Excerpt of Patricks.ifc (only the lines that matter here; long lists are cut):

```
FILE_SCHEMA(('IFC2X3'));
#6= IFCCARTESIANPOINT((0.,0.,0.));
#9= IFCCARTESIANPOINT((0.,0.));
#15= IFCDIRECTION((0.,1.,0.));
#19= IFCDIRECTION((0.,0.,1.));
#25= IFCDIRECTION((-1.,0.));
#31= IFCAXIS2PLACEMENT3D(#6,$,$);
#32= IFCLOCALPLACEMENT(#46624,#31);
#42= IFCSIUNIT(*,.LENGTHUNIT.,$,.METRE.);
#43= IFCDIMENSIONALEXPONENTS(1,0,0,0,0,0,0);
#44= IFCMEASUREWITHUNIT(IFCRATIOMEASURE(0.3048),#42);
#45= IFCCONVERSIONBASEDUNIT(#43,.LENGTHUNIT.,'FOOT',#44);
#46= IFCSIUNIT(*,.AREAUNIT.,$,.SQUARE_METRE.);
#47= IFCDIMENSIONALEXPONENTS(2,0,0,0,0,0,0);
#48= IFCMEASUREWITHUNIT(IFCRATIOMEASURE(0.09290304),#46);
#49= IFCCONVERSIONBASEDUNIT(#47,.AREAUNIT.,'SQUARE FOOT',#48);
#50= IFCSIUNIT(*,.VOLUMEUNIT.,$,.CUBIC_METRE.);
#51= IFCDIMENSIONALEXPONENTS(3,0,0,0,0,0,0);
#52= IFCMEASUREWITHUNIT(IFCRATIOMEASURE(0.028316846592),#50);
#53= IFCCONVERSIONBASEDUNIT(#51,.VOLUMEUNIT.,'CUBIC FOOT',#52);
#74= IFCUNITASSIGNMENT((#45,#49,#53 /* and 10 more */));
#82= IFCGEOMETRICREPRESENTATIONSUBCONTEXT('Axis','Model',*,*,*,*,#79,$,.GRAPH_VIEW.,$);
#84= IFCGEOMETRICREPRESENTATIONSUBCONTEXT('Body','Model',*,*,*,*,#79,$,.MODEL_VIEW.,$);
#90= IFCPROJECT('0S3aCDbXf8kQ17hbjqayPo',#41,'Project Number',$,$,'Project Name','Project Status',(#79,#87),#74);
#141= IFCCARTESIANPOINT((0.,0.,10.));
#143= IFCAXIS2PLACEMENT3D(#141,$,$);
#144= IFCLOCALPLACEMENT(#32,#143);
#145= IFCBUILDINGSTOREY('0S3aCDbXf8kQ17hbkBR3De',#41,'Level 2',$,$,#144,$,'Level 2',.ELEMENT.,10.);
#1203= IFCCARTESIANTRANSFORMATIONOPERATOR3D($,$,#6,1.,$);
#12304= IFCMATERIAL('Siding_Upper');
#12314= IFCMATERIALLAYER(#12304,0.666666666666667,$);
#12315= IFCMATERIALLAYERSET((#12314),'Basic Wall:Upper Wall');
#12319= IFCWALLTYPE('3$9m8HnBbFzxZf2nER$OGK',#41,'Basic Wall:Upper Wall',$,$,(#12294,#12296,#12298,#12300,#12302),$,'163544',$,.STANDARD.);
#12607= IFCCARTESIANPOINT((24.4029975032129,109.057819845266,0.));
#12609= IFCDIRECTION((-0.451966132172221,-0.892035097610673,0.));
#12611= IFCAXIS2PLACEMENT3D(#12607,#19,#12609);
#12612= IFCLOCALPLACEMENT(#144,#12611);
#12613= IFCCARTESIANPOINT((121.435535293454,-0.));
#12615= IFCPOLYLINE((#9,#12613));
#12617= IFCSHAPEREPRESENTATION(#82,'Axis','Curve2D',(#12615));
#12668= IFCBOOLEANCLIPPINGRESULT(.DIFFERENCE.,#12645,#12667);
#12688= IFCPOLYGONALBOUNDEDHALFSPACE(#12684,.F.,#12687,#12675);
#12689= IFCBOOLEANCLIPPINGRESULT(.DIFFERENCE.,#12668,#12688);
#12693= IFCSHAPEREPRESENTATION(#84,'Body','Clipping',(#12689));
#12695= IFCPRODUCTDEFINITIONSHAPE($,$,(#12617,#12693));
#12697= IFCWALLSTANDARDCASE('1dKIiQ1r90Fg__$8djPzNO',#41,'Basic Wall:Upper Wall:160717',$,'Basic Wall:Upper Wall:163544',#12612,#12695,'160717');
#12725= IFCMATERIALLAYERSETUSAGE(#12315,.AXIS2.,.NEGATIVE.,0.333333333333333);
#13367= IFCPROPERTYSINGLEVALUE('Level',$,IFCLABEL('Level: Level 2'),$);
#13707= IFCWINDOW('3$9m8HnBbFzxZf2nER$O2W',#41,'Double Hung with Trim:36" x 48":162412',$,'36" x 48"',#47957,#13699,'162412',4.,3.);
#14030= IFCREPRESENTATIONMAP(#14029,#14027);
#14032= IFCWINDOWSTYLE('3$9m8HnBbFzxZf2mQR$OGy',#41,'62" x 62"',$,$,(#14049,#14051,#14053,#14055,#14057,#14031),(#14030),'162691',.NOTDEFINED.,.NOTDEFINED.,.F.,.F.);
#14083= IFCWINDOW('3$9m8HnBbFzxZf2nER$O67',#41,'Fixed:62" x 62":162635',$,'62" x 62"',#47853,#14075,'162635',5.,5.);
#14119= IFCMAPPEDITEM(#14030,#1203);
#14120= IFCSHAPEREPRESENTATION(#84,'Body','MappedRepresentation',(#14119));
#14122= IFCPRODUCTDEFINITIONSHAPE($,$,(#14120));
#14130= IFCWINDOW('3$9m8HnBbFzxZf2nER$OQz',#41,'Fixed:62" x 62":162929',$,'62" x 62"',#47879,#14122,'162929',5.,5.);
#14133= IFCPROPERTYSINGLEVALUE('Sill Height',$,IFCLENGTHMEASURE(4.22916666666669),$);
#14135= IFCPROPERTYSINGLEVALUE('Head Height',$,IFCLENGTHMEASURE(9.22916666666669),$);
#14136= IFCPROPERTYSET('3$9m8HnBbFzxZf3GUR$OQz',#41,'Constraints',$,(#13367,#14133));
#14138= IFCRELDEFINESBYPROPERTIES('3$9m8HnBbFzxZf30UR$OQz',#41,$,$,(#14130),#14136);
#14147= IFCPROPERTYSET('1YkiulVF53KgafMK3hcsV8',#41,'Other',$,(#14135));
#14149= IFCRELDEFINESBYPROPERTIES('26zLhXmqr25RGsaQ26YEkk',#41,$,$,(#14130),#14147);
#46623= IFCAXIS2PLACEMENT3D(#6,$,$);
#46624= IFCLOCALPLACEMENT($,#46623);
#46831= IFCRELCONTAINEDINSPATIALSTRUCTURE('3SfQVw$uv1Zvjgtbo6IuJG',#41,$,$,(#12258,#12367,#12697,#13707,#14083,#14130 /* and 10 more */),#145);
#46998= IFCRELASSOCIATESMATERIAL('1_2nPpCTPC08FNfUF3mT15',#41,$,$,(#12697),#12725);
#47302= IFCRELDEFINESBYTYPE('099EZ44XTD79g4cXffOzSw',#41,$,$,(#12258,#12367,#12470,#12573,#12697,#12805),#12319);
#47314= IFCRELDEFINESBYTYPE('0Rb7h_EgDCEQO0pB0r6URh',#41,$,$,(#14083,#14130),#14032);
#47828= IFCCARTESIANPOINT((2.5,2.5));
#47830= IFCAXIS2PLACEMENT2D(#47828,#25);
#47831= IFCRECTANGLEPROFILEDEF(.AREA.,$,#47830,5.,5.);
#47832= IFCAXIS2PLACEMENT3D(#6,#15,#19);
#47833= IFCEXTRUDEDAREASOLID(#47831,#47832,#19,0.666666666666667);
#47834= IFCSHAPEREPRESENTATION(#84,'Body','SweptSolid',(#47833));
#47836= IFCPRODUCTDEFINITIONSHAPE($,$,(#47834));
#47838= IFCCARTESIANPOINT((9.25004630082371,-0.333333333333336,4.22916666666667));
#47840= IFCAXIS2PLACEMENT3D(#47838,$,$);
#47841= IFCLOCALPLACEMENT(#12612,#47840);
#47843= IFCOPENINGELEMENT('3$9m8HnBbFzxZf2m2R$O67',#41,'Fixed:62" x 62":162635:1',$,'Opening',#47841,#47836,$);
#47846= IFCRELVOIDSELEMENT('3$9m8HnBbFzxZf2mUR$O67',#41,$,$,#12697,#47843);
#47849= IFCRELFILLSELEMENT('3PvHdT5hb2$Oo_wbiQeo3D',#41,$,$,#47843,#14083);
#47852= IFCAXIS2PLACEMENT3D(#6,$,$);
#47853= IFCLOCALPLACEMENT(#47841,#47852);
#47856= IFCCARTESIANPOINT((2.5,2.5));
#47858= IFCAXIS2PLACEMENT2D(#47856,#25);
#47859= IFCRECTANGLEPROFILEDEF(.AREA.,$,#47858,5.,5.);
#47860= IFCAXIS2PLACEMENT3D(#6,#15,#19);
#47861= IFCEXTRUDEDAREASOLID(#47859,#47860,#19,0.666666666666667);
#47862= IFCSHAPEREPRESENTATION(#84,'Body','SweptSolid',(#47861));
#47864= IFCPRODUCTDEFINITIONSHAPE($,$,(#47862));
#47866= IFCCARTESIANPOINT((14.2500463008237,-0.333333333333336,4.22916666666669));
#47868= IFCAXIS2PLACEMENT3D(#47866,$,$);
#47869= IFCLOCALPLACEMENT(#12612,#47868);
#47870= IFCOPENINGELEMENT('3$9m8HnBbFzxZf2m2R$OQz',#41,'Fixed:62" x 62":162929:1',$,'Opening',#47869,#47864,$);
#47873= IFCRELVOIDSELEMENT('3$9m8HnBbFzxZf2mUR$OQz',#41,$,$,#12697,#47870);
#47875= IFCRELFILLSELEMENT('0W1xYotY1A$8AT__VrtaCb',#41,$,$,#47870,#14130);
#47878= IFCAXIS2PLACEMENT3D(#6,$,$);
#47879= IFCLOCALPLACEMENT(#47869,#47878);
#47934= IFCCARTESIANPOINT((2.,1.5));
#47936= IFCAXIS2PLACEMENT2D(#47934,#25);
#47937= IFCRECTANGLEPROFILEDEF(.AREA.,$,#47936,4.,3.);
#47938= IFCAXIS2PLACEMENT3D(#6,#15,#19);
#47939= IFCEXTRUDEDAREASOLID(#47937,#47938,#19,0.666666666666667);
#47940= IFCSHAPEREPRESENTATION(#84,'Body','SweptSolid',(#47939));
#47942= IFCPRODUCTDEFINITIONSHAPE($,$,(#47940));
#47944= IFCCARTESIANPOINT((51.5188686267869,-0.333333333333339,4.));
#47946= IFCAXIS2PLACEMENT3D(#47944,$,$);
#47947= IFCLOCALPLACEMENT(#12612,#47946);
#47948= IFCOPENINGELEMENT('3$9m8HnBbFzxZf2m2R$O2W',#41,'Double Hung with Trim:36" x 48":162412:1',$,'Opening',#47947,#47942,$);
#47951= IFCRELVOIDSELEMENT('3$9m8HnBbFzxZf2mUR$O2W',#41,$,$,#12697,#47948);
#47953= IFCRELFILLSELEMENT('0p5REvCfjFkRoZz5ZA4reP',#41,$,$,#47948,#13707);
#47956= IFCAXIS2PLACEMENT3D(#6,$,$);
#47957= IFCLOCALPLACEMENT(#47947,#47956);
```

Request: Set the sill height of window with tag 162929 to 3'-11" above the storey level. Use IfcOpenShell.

```python
import numpy as np
import ifcopenshell
import ifcopenshell.api.geometry
import ifcopenshell.api.pset
import ifcopenshell.geom
import ifcopenshell.util.element
import ifcopenshell.util.placement
import ifcopenshell.util.shape
import ifcopenshell.util.unit

model = ifcopenshell.open("Patricks.ifc")
unit_scale = ifcopenshell.util.unit.calculate_unit_scale(model)

window = model.by_guid("3$9m8HnBbFzxZf2nER$OQz")
opening = window.FillsVoids[0].RelatingOpeningElement
storey = ifcopenshell.util.element.get_container(window, ifc_class="IfcBuildingStorey")
level = ifcopenshell.util.placement.get_local_placement(storey.ObjectPlacement)[2, 3]

# The opening's origin need not be at the sill, so measure its lowest point.
shape = ifcopenshell.geom.create_shape(ifcopenshell.geom.settings(), opening)
bottom = ifcopenshell.util.shape.get_shape_bottom_elevation(shape, shape.geometry) / unit_scale
dz = level + 47 * 0.0254 / unit_scale - bottom

shift = np.array([0.0, 0.0, dz])
# The window is placed relative to its opening, so it follows when the opening moves.
matrix = ifcopenshell.util.placement.get_local_placement(opening.ObjectPlacement)
matrix[:3, 3] += shift
ifcopenshell.api.geometry.edit_object_placement(
    model, product=opening, matrix=matrix, is_si=False, should_transform_children=True
)

# Keep the stored heights in step.
pset = model.by_id(ifcopenshell.util.element.get_pset(window, "Constraints", should_inherit=False)["id"])
ifcopenshell.api.pset.edit_pset(model, pset=pset, properties={
    "Sill Height": model.create_entity("IfcLengthMeasure", ifcopenshell.util.element.get_pset(window, "Constraints", "Sill Height") + dz),
})
pset = model.by_id(ifcopenshell.util.element.get_pset(window, "Other", should_inherit=False)["id"])
ifcopenshell.api.pset.edit_pset(model, pset=pset, properties={
    "Head Height": model.create_entity("IfcLengthMeasure", ifcopenshell.util.element.get_pset(window, "Other", "Head Height") + dz),
})

print(f"moved by {dz * unit_scale:+.3f} m")

model.write("Patricks_rev.ifc")
```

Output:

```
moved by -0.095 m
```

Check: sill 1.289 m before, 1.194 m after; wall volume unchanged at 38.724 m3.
